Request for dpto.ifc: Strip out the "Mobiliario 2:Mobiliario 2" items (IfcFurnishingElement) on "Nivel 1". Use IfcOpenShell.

First a look at what the model holds.

```python
import ifcopenshell
import ifcopenshell.util.element

model = ifcopenshell.open("dpto.ifc")
print(model.schema)
storey = next(s for s in model.by_type("IfcBuildingStorey") if s.Name == "Nivel 1")
furniture = [e for e in ifcopenshell.util.element.get_decomposition(storey) if e.is_a("IfcFurnishingElement")]
seen = {}
for e in furniture:
    element_type = ifcopenshell.util.element.get_type(e)
    name = element_type.Name if element_type not in (None, e) else None
    seen[name] = seen.get(name, 0) + 1
for name, count in sorted(seen.items(), key=str):
    print(count, "x", name)
```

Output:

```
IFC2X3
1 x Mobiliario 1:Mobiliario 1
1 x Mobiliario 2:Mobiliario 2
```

```python
import ifcopenshell
import ifcopenshell.api.root
import ifcopenshell.util.element

model = ifcopenshell.open("dpto.ifc")

storey = next(s for s in model.by_type("IfcBuildingStorey") if s.Name == "Nivel 1")
furniture = [e for e in ifcopenshell.util.element.get_decomposition(storey) if e.is_a("IfcFurnishingElement")]
targets = [e for e in furniture if (t := ifcopenshell.util.element.get_type(e)) not in (None, e) and t.Name == "Mobiliario 2:Mobiliario 2"]

for e in targets:
    ifcopenshell.api.root.remove_product(model, product=e)
print(len(targets), "removed")

model.write("dpto_rev.ifc")
```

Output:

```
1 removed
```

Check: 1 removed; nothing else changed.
